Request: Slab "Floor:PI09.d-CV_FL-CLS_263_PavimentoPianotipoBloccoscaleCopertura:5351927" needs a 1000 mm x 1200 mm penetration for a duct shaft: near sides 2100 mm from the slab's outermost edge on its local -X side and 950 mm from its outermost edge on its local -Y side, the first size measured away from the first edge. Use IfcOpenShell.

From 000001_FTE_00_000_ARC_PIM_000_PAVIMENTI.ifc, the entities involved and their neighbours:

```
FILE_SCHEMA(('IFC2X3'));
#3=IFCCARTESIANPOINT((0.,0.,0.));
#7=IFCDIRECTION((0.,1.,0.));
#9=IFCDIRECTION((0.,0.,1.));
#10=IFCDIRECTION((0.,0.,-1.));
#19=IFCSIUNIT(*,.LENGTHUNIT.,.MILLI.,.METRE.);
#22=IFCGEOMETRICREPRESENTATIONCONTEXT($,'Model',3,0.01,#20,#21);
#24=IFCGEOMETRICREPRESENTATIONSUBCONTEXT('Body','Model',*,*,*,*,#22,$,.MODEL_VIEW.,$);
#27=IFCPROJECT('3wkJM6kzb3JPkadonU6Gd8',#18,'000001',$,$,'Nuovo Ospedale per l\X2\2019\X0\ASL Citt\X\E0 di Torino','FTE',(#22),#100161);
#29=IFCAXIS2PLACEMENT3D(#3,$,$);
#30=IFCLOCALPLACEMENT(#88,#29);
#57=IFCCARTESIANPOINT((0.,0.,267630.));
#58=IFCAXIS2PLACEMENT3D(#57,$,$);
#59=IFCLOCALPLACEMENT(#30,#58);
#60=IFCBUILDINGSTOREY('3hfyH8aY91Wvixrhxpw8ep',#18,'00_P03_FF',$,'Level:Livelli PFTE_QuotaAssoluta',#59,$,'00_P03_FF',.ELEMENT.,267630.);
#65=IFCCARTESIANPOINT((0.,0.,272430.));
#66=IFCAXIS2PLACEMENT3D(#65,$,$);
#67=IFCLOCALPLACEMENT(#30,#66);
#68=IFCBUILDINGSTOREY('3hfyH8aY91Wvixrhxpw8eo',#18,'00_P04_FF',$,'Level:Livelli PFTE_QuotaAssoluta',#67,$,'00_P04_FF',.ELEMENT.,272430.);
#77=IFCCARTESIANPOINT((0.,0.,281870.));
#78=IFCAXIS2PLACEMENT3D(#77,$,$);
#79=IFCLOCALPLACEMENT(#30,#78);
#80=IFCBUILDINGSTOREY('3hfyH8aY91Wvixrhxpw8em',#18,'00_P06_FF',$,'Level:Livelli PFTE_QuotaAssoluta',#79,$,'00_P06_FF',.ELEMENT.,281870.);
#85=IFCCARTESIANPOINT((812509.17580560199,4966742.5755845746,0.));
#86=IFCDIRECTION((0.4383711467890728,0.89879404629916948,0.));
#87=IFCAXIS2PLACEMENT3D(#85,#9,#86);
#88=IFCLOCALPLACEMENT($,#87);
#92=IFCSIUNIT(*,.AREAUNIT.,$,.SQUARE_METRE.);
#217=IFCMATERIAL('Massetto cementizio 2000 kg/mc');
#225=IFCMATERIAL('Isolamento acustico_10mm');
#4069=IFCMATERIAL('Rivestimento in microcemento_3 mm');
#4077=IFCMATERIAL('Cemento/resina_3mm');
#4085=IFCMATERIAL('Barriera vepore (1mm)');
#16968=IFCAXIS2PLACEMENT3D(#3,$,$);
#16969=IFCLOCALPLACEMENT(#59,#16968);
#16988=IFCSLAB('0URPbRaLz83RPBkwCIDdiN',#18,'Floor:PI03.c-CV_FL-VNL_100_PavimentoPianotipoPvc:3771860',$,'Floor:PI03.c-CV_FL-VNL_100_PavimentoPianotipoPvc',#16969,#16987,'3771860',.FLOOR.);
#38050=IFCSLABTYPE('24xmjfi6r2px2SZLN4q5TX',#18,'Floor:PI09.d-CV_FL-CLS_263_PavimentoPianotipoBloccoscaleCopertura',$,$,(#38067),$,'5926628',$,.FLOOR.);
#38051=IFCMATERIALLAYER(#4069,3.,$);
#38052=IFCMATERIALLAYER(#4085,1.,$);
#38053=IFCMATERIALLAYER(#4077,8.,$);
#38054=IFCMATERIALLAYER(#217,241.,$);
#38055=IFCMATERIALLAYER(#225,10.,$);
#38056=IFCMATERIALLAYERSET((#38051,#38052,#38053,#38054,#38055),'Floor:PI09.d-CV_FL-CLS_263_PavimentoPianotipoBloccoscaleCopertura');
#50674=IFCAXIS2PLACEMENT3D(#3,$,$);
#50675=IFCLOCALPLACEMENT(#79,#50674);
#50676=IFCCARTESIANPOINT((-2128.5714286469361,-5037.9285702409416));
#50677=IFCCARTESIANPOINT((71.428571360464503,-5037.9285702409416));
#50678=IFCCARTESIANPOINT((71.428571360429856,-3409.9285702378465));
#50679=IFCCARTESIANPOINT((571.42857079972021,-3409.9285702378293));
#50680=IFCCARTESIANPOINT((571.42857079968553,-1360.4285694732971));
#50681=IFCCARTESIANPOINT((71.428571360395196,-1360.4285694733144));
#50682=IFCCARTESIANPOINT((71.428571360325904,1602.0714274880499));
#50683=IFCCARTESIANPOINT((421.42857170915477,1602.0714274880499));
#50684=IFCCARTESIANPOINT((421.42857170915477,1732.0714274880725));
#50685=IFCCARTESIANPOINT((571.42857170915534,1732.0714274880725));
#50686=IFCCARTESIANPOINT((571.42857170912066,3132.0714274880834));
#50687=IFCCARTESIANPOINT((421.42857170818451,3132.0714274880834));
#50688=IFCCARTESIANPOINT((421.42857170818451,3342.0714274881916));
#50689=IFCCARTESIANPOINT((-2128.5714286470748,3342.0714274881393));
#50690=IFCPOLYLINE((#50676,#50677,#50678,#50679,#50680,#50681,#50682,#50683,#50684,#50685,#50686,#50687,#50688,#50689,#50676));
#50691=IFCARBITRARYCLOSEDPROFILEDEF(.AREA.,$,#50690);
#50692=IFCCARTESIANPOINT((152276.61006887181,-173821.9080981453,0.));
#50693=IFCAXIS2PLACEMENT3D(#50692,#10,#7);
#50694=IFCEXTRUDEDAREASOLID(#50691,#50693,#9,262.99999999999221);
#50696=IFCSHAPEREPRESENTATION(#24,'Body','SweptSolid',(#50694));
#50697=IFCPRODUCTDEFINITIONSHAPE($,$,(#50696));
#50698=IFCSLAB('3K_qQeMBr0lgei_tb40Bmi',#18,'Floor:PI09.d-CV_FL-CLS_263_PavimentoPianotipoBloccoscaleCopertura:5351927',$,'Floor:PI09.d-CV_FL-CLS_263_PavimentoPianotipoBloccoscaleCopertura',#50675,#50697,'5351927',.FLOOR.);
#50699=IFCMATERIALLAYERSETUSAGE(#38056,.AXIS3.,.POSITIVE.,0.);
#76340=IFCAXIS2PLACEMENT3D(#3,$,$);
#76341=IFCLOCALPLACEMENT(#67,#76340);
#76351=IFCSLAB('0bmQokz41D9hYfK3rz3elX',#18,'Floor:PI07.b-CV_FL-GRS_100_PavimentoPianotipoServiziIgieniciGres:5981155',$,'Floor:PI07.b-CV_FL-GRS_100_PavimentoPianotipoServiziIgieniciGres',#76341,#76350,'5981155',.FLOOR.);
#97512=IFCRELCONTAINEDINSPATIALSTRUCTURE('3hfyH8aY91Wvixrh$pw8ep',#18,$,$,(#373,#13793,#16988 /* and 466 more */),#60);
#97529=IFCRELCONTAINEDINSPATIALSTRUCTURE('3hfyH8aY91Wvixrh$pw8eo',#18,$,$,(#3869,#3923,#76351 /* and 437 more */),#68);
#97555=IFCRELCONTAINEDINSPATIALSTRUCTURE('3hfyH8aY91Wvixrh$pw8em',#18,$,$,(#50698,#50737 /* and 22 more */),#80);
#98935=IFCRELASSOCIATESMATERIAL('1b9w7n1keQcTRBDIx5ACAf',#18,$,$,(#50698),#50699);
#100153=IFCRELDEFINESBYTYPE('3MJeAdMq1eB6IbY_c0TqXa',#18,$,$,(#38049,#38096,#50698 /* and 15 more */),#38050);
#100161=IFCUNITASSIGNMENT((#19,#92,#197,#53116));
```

```python
import numpy as np
import ifcopenshell
import ifcopenshell.api.feature
import ifcopenshell.api.geometry
import ifcopenshell.api.root
import ifcopenshell.geom
import ifcopenshell.util.placement
import ifcopenshell.util.representation
import ifcopenshell.util.shape
import ifcopenshell.util.unit

model = ifcopenshell.open("000001_FTE_00_000_ARC_PIM_000_PAVIMENTI.ifc")
unit_scale = ifcopenshell.util.unit.calculate_unit_scale(model)
settings = ifcopenshell.geom.settings()


def volume(element):
    """Net volume in cubic metres, openings subtracted."""
    shape = ifcopenshell.geom.create_shape(settings, element)
    return ifcopenshell.util.shape.get_volume(shape.geometry)


slab = model.by_guid("3K_qQeMBr0lgei_tb40Bmi")
before = volume(slab)

# Extent in the slab's own axes, in metres. The edges named are its -X and -Y sides.
slab_shape = ifcopenshell.geom.create_shape(settings, slab)
vertices = ifcopenshell.util.shape.get_vertices(slab_shape.geometry)
x_min, y_min, bottom = vertices.min(axis=0)
top = vertices[:, 2].max()

opening = ifcopenshell.api.root.create_entity(model, ifc_class="IfcOpeningElement", name="Duct shaft opening")
context = ifcopenshell.util.representation.get_context(model, "Model", "Body", "MODEL_VIEW")
width, depth = 1, 1.2
outline = [(0.0, 0.0), (width, 0.0), (width, depth), (0.0, depth), (0.0, 0.0)]
# Overshoot both faces by 50 mm so the cut is clean.
shape = ifcopenshell.api.geometry.add_slab_representation(
    model, context=context, depth=top - bottom + 0.1, polyline=outline
)
ifcopenshell.api.geometry.assign_representation(model, product=opening, representation=shape)

matrix = ifcopenshell.util.placement.get_local_placement(slab.ObjectPlacement)
matrix[:, 3] = matrix @ np.append(np.array([x_min + 2.1, y_min + 0.95, bottom - 0.05]) / unit_scale, 1.0)
ifcopenshell.api.geometry.edit_object_placement(model, product=opening, matrix=matrix, is_si=False)
ifcopenshell.api.feature.add_feature(model, feature=opening, element=slab)

after = volume(slab)

print(f"slab volume {before:.3f} -> {after:.3f} m3")

model.write("000001_FTE_00_000_ARC_PIM_000_PAVIMENTI_updated.ifc")
```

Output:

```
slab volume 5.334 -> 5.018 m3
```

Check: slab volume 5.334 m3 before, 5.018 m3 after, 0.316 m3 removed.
